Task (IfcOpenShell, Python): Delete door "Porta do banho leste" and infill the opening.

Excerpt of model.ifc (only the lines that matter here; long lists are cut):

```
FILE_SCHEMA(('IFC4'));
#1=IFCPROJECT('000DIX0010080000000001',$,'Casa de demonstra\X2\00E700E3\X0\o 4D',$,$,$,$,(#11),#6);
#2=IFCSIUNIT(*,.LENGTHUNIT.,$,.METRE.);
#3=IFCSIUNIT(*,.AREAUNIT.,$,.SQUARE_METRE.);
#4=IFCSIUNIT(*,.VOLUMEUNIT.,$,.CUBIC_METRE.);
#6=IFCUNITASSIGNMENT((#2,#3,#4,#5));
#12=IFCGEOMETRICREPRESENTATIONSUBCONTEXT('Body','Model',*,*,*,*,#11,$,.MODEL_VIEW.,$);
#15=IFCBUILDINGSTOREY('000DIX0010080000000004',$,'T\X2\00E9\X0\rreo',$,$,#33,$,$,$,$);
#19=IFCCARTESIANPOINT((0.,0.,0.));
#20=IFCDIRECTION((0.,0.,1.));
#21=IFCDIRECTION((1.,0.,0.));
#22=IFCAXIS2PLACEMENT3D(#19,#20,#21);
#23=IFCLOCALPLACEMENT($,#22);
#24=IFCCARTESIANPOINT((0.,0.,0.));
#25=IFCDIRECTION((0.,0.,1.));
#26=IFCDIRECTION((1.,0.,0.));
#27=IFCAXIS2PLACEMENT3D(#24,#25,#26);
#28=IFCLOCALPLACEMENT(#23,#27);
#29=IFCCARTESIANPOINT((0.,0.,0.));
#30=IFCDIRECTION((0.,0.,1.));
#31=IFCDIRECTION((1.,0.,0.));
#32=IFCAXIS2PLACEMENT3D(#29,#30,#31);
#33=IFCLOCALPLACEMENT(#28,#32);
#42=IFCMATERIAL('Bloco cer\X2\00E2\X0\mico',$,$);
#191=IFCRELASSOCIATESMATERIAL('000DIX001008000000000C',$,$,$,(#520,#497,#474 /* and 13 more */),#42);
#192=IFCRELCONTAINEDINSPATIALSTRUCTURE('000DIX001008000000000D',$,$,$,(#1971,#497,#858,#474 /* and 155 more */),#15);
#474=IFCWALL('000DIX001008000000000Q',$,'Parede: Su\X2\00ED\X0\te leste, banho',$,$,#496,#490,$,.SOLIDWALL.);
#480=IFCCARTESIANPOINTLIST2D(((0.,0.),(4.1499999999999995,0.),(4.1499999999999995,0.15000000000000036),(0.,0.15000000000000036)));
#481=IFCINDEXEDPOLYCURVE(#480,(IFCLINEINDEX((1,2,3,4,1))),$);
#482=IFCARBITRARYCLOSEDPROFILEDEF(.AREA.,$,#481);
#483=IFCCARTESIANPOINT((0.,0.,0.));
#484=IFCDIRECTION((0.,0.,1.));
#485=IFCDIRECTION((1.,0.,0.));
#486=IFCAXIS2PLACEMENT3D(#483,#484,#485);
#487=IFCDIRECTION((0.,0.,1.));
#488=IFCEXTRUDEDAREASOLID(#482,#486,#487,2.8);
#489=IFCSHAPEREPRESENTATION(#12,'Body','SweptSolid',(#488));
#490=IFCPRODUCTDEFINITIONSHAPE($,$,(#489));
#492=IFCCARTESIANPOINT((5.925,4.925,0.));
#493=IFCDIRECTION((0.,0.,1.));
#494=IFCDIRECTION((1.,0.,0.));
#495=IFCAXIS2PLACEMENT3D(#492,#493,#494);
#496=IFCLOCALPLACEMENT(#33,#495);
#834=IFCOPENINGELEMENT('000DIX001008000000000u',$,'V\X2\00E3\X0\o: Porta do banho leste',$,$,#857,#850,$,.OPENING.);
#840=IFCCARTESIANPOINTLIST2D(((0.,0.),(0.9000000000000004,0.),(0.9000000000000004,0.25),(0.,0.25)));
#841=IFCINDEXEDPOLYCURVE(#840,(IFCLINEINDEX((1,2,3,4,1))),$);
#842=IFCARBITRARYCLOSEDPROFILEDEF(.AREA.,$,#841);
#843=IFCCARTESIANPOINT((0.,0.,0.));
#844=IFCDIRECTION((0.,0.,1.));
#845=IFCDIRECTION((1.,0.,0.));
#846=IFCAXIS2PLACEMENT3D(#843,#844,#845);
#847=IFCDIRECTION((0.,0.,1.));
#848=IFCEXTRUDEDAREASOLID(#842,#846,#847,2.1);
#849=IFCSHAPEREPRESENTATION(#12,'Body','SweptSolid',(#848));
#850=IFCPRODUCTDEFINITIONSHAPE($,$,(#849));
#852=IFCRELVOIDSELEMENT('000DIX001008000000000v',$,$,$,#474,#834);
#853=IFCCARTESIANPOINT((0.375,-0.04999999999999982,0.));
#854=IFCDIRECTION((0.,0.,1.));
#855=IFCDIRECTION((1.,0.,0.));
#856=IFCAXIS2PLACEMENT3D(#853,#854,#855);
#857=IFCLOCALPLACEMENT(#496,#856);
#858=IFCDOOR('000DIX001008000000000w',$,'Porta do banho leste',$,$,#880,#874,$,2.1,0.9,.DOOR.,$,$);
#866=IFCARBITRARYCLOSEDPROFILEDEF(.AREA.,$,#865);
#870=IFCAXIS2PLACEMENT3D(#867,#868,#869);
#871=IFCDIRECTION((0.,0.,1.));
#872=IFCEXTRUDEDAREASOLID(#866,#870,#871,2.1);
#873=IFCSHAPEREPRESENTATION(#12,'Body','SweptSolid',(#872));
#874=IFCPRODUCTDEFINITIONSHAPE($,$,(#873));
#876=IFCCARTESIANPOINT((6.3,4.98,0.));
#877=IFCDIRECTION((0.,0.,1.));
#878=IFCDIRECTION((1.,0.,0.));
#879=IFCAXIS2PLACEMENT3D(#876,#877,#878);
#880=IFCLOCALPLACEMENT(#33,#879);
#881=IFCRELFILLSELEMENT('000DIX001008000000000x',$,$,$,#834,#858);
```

```python
import ifcopenshell
import ifcopenshell.api.feature
import ifcopenshell.api.root
import ifcopenshell.geom
import ifcopenshell.util.shape

model = ifcopenshell.open("model.ifc")
settings = ifcopenshell.geom.settings()


def volume(element):
    """Net volume in cubic metres, openings subtracted."""
    shape = ifcopenshell.geom.create_shape(settings, element)
    return ifcopenshell.util.shape.get_volume(shape.geometry)


door = model.by_id(858)
opening = door.FillsVoids[0].RelatingOpeningElement
wall = opening.VoidsElements[0].RelatingBuildingElement
before = volume(wall)

ifcopenshell.api.root.remove_product(model, product=door)
ifcopenshell.api.feature.remove_feature(model, feature=opening)

after = volume(wall)

print(f"wall volume {before:.3f} -> {after:.3f} m3")

model.write("model_edited.ifc")
```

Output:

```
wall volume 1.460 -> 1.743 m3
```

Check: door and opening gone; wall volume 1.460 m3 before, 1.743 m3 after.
